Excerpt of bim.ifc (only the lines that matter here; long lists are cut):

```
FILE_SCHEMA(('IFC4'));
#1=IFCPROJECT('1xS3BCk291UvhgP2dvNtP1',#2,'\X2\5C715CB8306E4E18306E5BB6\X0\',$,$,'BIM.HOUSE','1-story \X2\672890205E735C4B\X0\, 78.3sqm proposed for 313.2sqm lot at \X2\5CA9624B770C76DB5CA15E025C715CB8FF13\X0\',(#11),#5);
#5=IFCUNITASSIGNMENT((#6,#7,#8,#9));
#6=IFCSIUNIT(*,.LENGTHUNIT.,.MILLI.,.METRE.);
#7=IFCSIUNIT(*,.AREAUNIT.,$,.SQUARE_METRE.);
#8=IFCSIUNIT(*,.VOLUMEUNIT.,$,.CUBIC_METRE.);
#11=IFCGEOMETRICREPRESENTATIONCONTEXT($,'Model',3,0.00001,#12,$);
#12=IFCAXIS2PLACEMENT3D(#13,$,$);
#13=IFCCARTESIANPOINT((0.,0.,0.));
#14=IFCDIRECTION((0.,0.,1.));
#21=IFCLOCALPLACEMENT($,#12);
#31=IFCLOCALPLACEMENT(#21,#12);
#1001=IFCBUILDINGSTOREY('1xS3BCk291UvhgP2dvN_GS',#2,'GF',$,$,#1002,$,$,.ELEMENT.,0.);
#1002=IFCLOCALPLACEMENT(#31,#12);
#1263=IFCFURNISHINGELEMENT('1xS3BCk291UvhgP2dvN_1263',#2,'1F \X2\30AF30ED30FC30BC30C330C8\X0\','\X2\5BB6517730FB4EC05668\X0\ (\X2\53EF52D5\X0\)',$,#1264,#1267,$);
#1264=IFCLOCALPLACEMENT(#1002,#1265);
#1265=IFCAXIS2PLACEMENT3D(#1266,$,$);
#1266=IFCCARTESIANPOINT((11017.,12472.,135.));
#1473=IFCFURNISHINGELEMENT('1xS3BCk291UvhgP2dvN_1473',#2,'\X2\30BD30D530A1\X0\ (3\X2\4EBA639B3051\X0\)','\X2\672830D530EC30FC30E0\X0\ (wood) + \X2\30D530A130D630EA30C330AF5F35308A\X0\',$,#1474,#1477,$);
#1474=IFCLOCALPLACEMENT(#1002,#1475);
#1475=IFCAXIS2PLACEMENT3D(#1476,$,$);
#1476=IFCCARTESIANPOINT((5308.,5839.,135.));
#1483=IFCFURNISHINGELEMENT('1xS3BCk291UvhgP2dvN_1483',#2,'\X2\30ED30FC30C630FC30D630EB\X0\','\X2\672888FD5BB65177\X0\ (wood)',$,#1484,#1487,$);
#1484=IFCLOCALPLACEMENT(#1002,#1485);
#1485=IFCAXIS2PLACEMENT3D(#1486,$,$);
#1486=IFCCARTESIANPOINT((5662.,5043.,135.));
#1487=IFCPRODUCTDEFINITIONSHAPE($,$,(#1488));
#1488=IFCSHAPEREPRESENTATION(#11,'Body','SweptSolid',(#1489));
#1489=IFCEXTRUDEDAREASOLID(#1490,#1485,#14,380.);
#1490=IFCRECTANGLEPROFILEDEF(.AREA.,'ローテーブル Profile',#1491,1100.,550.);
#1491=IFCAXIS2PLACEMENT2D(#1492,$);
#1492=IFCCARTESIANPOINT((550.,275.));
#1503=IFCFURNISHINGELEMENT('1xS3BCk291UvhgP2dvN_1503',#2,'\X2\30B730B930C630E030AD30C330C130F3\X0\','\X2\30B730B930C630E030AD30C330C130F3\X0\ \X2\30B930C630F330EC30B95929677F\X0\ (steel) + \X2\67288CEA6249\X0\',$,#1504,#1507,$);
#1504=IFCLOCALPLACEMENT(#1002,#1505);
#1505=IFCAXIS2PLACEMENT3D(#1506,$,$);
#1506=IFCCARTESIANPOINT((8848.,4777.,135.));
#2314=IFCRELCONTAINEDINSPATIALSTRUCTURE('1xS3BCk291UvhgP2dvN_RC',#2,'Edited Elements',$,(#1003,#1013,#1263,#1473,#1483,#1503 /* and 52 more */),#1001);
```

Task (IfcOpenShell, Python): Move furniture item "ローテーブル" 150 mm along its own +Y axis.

```python
import ifcopenshell
import ifcopenshell.api.geometry
import ifcopenshell.util.placement

model = ifcopenshell.open("bim.ifc")

item = model.by_guid("1xS3BCk291UvhgP2dvN_1483")
matrix = ifcopenshell.util.placement.get_local_placement(item.ObjectPlacement)
matrix[:3, 3] += matrix[:3, 1] * 150.0
ifcopenshell.api.geometry.edit_object_placement(model, product=item, matrix=matrix, is_si=False)

print(ifcopenshell.util.placement.get_local_placement(item.ObjectPlacement).round(3) + 0.0)

model.write("bim_rev.ifc")
```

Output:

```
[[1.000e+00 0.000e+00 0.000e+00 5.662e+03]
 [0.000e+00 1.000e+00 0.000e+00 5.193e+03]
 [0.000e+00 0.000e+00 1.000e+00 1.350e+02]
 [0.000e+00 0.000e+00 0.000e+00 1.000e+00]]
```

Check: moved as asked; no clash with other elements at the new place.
